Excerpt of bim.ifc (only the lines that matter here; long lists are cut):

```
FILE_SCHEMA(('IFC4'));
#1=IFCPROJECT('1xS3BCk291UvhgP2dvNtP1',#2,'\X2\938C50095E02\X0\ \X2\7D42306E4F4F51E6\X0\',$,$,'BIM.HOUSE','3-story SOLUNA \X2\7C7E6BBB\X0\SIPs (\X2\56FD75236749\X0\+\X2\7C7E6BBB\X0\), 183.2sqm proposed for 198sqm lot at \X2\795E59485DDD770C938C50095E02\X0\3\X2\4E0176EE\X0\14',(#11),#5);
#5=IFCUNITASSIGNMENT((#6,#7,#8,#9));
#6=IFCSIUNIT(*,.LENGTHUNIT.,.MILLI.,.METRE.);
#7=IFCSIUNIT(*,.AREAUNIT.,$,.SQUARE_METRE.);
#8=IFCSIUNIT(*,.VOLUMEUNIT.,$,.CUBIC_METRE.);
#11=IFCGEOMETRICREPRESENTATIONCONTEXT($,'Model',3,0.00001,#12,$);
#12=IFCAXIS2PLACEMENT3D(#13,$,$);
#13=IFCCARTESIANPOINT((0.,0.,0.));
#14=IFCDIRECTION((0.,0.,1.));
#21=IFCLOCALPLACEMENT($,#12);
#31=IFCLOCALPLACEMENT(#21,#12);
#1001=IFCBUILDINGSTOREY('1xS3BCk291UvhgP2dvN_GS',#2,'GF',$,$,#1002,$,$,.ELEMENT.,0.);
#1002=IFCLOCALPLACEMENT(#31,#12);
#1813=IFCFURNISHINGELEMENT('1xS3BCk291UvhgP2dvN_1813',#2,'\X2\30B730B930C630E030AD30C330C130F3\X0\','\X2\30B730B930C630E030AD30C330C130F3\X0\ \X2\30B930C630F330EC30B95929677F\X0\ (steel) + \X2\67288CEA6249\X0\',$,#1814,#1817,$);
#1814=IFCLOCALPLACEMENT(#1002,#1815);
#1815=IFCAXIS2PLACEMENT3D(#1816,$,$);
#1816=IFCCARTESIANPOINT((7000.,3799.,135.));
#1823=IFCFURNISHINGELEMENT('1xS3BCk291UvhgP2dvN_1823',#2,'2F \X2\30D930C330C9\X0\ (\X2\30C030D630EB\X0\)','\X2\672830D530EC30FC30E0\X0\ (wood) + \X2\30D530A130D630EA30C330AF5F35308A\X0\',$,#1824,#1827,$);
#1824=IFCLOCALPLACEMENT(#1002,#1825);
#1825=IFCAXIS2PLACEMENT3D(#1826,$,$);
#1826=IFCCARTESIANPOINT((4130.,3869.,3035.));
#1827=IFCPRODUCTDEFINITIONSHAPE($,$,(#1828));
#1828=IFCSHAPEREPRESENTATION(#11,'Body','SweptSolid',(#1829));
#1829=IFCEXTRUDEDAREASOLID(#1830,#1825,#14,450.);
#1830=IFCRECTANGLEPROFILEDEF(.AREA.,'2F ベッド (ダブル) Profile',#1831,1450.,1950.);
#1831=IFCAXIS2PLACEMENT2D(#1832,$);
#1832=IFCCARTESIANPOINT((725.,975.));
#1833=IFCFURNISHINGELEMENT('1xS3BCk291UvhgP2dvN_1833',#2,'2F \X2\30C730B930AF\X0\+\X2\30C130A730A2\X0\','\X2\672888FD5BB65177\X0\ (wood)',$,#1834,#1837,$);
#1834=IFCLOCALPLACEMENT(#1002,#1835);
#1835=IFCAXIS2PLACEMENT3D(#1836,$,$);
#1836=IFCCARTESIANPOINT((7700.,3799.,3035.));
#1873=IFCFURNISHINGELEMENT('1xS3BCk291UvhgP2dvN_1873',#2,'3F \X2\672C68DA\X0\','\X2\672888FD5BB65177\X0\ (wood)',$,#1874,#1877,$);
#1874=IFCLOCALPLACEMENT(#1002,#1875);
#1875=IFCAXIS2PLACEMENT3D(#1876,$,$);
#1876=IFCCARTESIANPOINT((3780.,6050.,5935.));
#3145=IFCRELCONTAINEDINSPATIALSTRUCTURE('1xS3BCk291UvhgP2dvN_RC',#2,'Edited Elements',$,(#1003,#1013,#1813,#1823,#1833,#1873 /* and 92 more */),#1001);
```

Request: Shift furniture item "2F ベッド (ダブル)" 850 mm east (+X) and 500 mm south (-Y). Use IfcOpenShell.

```python
import ifcopenshell
import ifcopenshell.api.geometry
import ifcopenshell.util.placement
import ifcopenshell.util.unit

model = ifcopenshell.open("bim.ifc")
unit_scale = ifcopenshell.util.unit.calculate_unit_scale(model)

item = model.by_id(1823)
matrix = ifcopenshell.util.placement.get_local_placement(item.ObjectPlacement)
matrix[0, 3] += 0.85 / unit_scale
matrix[1, 3] -= 0.5 / unit_scale
ifcopenshell.api.geometry.edit_object_placement(model, product=item, matrix=matrix, is_si=False)

print(ifcopenshell.util.placement.get_local_placement(item.ObjectPlacement).round(3) + 0.0)

model.write("bim_rev.ifc")
```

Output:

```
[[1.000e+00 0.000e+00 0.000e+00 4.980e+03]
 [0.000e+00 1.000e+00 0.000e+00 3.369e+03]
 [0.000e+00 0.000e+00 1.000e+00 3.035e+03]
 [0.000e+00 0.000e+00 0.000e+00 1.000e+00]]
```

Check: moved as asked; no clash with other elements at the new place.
